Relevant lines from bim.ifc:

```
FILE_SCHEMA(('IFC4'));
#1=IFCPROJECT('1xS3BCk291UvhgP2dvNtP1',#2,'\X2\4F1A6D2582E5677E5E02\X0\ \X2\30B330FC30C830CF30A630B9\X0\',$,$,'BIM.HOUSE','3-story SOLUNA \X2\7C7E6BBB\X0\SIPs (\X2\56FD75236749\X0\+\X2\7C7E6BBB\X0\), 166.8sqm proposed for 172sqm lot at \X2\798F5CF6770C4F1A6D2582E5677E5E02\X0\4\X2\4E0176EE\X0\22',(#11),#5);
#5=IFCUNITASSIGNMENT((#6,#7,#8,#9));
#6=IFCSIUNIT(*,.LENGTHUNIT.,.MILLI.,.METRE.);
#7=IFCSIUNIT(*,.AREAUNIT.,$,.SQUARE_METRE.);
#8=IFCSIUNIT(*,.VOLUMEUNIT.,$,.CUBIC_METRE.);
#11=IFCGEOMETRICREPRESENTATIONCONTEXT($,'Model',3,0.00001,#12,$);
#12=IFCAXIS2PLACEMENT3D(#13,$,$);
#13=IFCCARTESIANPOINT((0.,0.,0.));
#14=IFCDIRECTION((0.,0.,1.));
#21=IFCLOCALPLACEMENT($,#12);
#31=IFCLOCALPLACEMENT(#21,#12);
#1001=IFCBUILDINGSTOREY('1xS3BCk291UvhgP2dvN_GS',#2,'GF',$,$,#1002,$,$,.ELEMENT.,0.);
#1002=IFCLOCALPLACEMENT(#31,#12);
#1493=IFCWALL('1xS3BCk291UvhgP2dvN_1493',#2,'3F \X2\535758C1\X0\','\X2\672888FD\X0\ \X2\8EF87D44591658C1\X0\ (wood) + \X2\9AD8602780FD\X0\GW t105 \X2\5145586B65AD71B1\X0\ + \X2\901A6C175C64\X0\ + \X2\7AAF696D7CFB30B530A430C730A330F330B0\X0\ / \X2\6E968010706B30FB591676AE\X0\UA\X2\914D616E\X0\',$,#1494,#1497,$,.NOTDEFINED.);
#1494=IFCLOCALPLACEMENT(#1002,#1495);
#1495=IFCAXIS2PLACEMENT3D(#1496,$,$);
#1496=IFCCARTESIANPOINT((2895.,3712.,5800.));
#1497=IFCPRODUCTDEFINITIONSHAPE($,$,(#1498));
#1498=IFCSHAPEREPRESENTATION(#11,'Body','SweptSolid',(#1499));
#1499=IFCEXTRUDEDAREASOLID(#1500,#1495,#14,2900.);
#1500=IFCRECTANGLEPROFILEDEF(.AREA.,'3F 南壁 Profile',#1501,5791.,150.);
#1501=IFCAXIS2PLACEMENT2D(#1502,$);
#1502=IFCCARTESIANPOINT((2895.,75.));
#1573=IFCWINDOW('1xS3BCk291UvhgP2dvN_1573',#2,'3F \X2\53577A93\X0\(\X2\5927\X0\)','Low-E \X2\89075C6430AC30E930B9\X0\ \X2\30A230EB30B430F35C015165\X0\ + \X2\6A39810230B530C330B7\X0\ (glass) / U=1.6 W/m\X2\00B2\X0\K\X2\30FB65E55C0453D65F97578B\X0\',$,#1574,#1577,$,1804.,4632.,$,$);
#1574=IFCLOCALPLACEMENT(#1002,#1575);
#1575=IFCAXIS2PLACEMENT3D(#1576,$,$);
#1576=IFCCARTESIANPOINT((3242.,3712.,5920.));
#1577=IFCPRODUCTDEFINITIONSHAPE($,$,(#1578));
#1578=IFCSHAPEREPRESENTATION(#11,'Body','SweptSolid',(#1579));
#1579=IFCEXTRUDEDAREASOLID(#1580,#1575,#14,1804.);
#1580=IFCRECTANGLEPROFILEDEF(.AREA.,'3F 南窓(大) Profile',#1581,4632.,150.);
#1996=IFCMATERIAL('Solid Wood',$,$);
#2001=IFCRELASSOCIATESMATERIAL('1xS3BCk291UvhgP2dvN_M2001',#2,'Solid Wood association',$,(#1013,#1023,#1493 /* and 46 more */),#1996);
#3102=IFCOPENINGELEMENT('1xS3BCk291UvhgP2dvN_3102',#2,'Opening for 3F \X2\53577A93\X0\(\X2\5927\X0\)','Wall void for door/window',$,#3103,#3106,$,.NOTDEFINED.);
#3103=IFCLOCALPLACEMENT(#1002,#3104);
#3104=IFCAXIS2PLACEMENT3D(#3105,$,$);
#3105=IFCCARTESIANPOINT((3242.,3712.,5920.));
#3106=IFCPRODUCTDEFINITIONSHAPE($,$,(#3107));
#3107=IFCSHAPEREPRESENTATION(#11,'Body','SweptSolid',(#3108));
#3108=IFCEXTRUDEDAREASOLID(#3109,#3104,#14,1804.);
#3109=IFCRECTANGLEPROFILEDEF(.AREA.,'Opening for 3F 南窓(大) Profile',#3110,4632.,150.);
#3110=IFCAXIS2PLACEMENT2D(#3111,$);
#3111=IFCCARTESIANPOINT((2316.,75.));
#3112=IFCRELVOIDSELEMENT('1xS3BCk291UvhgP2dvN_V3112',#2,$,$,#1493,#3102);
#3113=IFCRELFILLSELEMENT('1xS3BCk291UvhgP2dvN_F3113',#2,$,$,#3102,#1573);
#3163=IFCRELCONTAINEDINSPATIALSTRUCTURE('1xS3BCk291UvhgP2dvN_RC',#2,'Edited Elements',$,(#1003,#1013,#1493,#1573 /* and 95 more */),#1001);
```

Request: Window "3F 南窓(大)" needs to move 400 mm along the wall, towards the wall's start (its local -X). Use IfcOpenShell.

```python
import ifcopenshell
import ifcopenshell.api.geometry
import ifcopenshell.util.placement

model = ifcopenshell.open("bim.ifc")

window = model.by_guid("1xS3BCk291UvhgP2dvN_1573")
opening = window.FillsVoids[0].RelatingOpeningElement
wall = opening.VoidsElements[0].RelatingBuildingElement

wall_matrix = ifcopenshell.util.placement.get_local_placement(wall.ObjectPlacement)
shift = wall_matrix[:3, 0] * -400.0
before = ifcopenshell.util.placement.get_local_placement(window.ObjectPlacement)[:3, 3].copy()

# The window is not placed relative to its opening, so move both.
for product in (opening, window):
    matrix = ifcopenshell.util.placement.get_local_placement(product.ObjectPlacement)
    matrix[:3, 3] += shift
    ifcopenshell.api.geometry.edit_object_placement(model, product=product, matrix=matrix, is_si=False)

after = ifcopenshell.util.placement.get_local_placement(window.ObjectPlacement)[:3, 3]
print("window moved by", (after - before).round(3) + 0.0)

model.write("bim_updated.ifc")
```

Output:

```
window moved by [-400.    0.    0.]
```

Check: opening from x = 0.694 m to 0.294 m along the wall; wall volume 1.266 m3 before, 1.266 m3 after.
